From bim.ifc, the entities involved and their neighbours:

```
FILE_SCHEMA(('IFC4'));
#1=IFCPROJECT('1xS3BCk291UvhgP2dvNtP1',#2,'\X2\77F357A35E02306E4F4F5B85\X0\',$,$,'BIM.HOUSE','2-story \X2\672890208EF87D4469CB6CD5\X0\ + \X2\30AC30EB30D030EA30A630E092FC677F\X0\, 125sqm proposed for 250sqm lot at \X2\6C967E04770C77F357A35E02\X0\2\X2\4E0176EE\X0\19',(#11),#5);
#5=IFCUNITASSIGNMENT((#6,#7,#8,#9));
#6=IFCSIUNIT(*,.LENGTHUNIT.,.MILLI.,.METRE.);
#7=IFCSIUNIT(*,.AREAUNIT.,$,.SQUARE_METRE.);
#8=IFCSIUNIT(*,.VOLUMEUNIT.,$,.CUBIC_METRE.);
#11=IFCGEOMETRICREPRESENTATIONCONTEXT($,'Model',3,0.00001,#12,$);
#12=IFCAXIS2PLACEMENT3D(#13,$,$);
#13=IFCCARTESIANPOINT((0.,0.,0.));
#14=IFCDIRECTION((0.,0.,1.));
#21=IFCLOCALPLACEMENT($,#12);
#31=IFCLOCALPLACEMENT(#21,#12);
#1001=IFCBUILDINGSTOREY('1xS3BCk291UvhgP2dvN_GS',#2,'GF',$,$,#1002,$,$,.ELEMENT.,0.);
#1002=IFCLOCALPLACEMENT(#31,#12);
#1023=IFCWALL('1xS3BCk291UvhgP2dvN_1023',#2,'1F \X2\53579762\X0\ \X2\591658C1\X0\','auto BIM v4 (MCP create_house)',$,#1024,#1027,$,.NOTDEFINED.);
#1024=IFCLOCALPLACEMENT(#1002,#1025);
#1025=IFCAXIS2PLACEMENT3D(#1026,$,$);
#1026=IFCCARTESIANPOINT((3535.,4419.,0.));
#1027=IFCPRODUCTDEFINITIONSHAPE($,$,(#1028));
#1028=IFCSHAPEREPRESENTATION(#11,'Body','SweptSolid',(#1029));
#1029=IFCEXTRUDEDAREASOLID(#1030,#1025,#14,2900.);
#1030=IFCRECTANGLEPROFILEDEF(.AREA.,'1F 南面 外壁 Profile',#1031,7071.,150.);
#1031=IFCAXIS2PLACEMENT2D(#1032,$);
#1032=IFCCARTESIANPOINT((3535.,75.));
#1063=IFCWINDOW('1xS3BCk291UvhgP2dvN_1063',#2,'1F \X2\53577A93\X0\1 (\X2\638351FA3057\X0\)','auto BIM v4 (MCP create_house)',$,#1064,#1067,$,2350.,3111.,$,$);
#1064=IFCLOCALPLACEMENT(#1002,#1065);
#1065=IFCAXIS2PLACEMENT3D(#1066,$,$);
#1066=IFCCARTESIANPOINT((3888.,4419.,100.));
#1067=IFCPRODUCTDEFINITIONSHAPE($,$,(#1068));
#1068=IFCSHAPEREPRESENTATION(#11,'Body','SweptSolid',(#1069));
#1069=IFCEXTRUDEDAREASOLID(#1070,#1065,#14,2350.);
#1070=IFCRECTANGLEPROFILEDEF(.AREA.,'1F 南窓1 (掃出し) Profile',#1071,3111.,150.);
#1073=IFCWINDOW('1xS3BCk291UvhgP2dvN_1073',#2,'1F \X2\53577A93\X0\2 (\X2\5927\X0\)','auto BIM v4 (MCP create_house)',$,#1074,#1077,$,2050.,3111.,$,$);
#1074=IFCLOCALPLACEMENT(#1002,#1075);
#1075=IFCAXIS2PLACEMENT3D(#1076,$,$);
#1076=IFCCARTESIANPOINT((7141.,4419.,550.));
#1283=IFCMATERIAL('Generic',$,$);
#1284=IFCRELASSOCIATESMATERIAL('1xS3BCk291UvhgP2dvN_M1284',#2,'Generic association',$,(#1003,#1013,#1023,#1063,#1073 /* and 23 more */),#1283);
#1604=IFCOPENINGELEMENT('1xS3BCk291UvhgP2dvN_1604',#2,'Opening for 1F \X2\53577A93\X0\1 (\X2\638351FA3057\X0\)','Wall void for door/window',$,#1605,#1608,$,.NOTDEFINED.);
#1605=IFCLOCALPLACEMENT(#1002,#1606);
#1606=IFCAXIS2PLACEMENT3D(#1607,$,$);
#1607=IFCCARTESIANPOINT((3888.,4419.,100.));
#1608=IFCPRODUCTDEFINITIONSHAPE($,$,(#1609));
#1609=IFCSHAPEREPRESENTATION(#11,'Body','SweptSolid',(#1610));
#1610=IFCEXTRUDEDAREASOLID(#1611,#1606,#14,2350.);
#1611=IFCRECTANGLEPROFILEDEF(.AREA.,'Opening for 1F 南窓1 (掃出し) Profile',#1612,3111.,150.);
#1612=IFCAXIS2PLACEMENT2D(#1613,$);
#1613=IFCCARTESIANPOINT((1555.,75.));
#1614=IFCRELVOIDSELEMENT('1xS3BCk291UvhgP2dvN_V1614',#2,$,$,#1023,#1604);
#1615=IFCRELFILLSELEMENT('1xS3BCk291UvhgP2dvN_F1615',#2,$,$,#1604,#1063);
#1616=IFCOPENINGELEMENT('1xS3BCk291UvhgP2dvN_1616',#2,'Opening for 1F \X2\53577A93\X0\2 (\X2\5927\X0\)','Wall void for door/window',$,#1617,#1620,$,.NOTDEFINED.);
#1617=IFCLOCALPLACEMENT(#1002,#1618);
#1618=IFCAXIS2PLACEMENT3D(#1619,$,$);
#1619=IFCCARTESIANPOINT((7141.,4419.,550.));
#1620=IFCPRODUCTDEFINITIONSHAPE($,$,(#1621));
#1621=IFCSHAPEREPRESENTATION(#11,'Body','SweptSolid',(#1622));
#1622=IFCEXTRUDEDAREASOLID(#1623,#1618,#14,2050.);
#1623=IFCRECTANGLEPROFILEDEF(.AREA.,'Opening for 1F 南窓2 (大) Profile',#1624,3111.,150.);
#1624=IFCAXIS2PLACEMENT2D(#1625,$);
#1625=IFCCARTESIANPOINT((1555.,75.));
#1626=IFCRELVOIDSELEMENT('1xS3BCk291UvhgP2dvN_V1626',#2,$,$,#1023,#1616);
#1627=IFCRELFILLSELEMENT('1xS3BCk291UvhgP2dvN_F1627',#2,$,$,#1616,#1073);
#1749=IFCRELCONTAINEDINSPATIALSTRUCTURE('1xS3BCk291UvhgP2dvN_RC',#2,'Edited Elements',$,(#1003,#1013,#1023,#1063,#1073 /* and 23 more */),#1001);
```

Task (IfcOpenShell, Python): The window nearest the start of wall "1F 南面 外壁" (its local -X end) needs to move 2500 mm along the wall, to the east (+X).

```python
import ifcopenshell
import ifcopenshell.api.geometry
import ifcopenshell.util.placement

model = ifcopenshell.open("bim.ifc")

window = model.by_guid("1xS3BCk291UvhgP2dvN_1063")
opening = window.FillsVoids[0].RelatingOpeningElement
wall = opening.VoidsElements[0].RelatingBuildingElement

wall_matrix = ifcopenshell.util.placement.get_local_placement(wall.ObjectPlacement)
shift = wall_matrix[:3, 0] * 2500.0
before = ifcopenshell.util.placement.get_local_placement(window.ObjectPlacement)[:3, 3].copy()

# The window is not placed relative to its opening, so move both.
for product in (opening, window):
    matrix = ifcopenshell.util.placement.get_local_placement(product.ObjectPlacement)
    matrix[:3, 3] += shift
    ifcopenshell.api.geometry.edit_object_placement(model, product=product, matrix=matrix, is_si=False)

after = ifcopenshell.util.placement.get_local_placement(window.ObjectPlacement)[:3, 3]
print("window moved by", (after - before).round(3) + 0.0)

model.write("bim-out.ifc")
```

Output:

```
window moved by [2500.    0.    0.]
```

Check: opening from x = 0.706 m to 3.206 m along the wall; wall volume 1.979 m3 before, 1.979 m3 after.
